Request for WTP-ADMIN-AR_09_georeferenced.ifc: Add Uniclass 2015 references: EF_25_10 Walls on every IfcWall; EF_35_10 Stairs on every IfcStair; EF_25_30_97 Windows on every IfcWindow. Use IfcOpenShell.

First a look at what the model holds.

```python
import ifcopenshell

model = ifcopenshell.open("WTP-ADMIN-AR_09_georeferenced.ifc")
print(model.schema)
print("classifications:", [c.Name for c in model.by_type("IfcClassification")])
for ifc_class in ("IfcDoor", "IfcRoof", "IfcStair", "IfcWall", "IfcWindow"):
    print(ifc_class, len(model.by_type(ifc_class)))
```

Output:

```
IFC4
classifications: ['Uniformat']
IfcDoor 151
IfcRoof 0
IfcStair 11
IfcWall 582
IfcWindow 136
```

```python
import ifcopenshell
import ifcopenshell.api.classification

model = ifcopenshell.open("WTP-ADMIN-AR_09_georeferenced.ifc")

system = ifcopenshell.api.classification.add_classification(model, classification="Uniclass 2015")

codes = {
    "IfcWall": ("EF_25_10", "Walls"),
    "IfcStair": ("EF_35_10", "Stairs"),
    "IfcWindow": ("EF_25_30_97", "Windows"),
}
for ifc_class, (code, name) in codes.items():
    products = model.by_type(ifc_class)
    ifcopenshell.api.classification.add_reference(
        model, products=products, classification=system, identification=code, name=name
    )
    print(code, len(products))

model.write("WTP-ADMIN-AR_09_georeferenced_v2.ifc")
```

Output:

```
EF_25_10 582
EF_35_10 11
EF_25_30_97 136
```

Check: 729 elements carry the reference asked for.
